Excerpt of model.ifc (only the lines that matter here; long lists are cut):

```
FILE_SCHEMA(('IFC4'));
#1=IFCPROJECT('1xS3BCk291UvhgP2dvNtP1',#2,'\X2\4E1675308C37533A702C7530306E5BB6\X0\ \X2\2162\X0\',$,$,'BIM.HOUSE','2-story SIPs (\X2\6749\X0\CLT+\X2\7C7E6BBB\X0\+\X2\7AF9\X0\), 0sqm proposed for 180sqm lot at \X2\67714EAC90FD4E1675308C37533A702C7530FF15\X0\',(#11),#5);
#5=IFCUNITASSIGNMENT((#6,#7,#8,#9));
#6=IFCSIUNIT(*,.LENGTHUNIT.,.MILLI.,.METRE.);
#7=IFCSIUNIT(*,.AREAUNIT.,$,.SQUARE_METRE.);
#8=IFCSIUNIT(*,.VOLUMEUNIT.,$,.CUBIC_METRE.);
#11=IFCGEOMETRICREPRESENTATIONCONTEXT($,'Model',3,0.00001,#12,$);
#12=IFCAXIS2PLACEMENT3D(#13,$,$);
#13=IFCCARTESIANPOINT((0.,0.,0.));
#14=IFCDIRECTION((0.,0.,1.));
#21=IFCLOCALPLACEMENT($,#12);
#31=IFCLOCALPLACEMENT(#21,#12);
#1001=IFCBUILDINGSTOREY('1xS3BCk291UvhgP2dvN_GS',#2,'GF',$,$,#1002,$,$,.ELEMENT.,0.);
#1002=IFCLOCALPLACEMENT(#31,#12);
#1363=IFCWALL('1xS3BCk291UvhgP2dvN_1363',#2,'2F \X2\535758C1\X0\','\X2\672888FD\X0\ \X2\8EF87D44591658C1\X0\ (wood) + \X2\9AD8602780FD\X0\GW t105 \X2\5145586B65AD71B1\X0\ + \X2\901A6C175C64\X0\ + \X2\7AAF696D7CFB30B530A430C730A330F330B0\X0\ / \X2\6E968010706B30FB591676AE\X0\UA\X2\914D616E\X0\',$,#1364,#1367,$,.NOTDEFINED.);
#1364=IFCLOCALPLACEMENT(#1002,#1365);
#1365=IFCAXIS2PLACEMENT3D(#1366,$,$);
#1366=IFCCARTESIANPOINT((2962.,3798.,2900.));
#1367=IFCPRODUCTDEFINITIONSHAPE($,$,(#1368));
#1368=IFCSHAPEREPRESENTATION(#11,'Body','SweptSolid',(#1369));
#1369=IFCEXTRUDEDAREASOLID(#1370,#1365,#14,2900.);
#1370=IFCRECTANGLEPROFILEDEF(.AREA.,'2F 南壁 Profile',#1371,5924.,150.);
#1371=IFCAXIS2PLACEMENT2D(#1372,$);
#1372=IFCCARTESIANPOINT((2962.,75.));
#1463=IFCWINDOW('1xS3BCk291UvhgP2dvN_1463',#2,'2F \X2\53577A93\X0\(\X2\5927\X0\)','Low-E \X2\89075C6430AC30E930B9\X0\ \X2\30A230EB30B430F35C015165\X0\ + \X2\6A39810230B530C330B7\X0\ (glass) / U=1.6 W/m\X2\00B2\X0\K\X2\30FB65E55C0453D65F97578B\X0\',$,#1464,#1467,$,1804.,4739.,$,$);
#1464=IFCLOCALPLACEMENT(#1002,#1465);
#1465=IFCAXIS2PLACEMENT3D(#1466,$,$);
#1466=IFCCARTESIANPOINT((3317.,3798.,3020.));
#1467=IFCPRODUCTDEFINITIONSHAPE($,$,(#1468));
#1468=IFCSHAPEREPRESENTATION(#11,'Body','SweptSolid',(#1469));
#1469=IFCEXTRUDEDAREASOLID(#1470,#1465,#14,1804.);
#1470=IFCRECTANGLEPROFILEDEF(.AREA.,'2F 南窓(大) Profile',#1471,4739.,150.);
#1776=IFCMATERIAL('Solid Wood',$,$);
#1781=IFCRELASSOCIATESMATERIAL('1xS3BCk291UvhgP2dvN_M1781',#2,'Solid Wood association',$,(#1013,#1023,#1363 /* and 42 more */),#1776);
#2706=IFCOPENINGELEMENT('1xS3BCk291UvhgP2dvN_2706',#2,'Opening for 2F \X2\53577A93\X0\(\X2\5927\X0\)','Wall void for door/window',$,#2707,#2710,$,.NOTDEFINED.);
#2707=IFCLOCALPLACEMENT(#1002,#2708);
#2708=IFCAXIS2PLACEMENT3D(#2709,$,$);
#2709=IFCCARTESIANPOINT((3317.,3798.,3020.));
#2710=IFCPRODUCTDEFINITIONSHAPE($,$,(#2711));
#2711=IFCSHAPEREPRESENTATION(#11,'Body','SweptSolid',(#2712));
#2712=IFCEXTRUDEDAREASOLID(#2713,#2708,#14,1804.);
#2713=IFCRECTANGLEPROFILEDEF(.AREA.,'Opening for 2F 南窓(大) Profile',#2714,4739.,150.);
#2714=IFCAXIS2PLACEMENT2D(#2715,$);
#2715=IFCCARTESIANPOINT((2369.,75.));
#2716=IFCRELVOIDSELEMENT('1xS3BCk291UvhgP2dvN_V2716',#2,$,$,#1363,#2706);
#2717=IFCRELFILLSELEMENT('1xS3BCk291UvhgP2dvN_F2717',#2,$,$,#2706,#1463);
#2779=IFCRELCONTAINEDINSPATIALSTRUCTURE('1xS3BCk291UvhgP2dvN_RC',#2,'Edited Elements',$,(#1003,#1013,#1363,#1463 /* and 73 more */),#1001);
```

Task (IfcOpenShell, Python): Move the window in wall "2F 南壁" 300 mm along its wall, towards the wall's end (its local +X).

```python
import ifcopenshell
import ifcopenshell.api.geometry
import ifcopenshell.util.placement

model = ifcopenshell.open("model.ifc")

window = model.by_guid("1xS3BCk291UvhgP2dvN_1463")
opening = window.FillsVoids[0].RelatingOpeningElement
wall = opening.VoidsElements[0].RelatingBuildingElement

wall_matrix = ifcopenshell.util.placement.get_local_placement(wall.ObjectPlacement)
shift = wall_matrix[:3, 0] * 300.0
before = ifcopenshell.util.placement.get_local_placement(window.ObjectPlacement)[:3, 3].copy()

# The window is not placed relative to its opening, so move both.
for product in (opening, window):
    matrix = ifcopenshell.util.placement.get_local_placement(product.ObjectPlacement)
    matrix[:3, 3] += shift
    ifcopenshell.api.geometry.edit_object_placement(model, product=product, matrix=matrix, is_si=False)

after = ifcopenshell.util.placement.get_local_placement(window.ObjectPlacement)[:3, 3]
print("window moved by", (after - before).round(3) + 0.0)

model.write("model-out.ifc")
```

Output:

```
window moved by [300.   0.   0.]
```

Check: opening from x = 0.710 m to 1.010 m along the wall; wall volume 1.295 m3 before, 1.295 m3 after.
